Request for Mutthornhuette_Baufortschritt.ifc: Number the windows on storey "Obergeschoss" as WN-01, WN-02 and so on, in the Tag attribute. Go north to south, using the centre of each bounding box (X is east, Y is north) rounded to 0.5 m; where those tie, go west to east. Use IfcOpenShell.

First a look at what the model holds.

```python
import ifcopenshell
import ifcopenshell.util.element
import ifcopenshell.util.placement

model = ifcopenshell.open("Mutthornhuette_Baufortschritt.ifc")
print(model.schema)
storey = next(s for s in model.by_type("IfcBuildingStorey") if s.Name == "Obergeschoss")
windows = [e for e in ifcopenshell.util.element.get_decomposition(storey) if e.is_a("IfcWindow")]
for e in sorted(windows, key=lambda e: e.id()):
    origin = ifcopenshell.util.placement.get_local_placement(e.ObjectPlacement)[:3, 3]
    print(e.id(), e.Tag, e.Name, origin.round(2) + 0.0, sep=" | ")
```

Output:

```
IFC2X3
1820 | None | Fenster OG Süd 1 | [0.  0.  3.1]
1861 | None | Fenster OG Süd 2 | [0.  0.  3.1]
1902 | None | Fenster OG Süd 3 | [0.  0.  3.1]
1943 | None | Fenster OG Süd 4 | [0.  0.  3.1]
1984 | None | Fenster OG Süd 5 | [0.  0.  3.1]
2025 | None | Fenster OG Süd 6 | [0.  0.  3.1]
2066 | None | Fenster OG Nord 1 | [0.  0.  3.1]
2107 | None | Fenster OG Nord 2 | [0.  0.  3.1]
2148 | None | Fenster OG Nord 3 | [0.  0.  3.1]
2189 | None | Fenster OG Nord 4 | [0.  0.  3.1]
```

```python
import ifcopenshell
import ifcopenshell.geom
import ifcopenshell.util.element
import ifcopenshell.util.shape

model = ifcopenshell.open("Mutthornhuette_Baufortschritt.ifc")
settings = ifcopenshell.geom.settings()
settings.set("use-world-coords", True)


def centre(element):
    shape = ifcopenshell.geom.create_shape(settings, element)
    return ifcopenshell.util.shape.get_bbox_centroid(shape.geometry)


storey = next(s for s in model.by_type("IfcBuildingStorey") if s.Name == "Obergeschoss")
windows = [e for e in ifcopenshell.util.element.get_decomposition(storey) if e.is_a("IfcWindow")]

# Insertion points can sit at a corner or the storey origin, so sort by the geometry (in metres).
centres = {e: centre(e) for e in windows}
windows.sort(key=lambda e: (-round(centres[e][1] / 0.5), centres[e][0]))

for i, e in enumerate(windows, start=1):
    number = f"WN-{i:02d}"
    e.Tag = number
    print(e.id(), number)

model.write("Mutthornhuette_Baufortschritt_edited.ifc")
```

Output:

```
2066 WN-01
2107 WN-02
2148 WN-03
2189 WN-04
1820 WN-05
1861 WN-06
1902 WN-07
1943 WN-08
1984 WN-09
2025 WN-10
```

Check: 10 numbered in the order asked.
